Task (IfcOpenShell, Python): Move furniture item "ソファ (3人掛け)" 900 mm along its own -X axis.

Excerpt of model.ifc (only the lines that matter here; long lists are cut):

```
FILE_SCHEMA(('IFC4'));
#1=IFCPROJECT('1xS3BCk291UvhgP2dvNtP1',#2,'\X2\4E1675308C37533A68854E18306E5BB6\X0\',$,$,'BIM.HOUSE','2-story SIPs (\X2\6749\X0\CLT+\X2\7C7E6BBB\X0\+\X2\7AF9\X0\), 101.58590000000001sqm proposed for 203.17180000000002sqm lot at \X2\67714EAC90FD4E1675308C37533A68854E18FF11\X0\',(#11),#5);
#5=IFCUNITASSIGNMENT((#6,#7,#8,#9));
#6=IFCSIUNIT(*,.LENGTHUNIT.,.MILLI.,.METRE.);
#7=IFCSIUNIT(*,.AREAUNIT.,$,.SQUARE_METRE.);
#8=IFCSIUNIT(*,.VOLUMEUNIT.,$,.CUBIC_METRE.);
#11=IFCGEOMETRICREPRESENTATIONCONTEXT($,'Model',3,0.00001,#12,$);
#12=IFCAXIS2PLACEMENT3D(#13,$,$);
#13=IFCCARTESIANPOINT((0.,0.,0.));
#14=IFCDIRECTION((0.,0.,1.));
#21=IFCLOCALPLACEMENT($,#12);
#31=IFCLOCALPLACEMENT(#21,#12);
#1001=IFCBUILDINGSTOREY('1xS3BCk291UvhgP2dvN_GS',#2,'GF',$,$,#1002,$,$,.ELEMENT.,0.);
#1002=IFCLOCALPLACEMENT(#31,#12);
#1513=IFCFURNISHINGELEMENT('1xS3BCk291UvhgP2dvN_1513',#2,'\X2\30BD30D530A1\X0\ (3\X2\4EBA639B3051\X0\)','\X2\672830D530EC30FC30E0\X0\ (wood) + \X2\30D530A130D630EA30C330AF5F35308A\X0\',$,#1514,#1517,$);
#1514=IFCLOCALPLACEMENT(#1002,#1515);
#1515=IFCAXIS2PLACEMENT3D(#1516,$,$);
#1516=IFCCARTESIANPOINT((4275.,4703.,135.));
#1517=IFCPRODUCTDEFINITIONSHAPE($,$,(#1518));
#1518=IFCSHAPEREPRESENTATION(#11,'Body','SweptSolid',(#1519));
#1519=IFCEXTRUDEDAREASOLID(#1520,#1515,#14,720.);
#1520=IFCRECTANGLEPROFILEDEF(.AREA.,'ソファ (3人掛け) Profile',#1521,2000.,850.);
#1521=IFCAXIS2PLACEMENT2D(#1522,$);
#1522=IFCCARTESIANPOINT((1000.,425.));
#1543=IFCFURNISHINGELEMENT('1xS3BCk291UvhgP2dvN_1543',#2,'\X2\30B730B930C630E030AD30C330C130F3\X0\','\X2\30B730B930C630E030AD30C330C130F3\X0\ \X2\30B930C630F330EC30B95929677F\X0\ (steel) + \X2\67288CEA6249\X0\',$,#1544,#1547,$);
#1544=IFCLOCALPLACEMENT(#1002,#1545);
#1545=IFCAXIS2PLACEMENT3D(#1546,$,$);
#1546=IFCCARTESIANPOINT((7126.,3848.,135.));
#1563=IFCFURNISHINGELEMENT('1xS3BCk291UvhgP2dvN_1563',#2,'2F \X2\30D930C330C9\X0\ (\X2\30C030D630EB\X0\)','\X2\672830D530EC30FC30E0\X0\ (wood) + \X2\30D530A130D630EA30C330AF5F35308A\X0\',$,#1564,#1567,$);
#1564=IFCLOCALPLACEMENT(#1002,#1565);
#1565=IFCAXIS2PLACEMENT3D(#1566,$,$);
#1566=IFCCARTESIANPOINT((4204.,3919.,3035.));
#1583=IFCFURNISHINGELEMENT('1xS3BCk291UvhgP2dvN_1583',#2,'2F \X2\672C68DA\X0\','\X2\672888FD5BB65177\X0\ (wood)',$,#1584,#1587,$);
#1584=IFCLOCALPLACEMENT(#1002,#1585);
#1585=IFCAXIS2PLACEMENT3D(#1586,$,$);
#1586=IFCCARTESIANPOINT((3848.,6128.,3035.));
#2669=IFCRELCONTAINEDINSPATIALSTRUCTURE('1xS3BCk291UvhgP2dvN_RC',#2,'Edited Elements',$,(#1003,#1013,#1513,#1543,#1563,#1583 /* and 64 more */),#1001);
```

```python
import ifcopenshell
import ifcopenshell.api.geometry
import ifcopenshell.util.placement
import ifcopenshell.util.unit

model = ifcopenshell.open("model.ifc")
unit_scale = ifcopenshell.util.unit.calculate_unit_scale(model)

item = model.by_id(1513)
matrix = ifcopenshell.util.placement.get_local_placement(item.ObjectPlacement)
matrix[:3, 3] -= matrix[:3, 0] * 0.9 / unit_scale
ifcopenshell.api.geometry.edit_object_placement(model, product=item, matrix=matrix, is_si=False)

print(ifcopenshell.util.placement.get_local_placement(item.ObjectPlacement).round(3) + 0.0)

model.write("model-out.ifc")
```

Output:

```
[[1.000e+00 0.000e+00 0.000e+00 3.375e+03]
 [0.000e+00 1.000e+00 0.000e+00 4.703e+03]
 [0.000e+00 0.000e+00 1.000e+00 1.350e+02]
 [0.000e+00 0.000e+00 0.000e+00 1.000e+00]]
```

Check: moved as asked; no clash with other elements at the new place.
